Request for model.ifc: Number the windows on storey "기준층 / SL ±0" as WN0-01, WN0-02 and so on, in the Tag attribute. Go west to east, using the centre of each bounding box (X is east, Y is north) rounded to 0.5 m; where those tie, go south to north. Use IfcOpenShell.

First a look at what the model holds.

```python
import ifcopenshell
import ifcopenshell.util.element
import ifcopenshell.util.placement

model = ifcopenshell.open("model.ifc")
print(model.schema)
storey = next(s for s in model.by_type("IfcBuildingStorey") if s.Name == "기준층 / SL ±0")
windows = [e for e in ifcopenshell.util.element.get_decomposition(storey) if e.is_a("IfcWindow")]
for e in sorted(windows, key=lambda e: e.id()):
    origin = ifcopenshell.util.placement.get_local_placement(e.ObjectPlacement)[:3, 3]
    print(e.id(), e.Tag, e.Name, origin.round(2) + 0.0, sep=" | ")
```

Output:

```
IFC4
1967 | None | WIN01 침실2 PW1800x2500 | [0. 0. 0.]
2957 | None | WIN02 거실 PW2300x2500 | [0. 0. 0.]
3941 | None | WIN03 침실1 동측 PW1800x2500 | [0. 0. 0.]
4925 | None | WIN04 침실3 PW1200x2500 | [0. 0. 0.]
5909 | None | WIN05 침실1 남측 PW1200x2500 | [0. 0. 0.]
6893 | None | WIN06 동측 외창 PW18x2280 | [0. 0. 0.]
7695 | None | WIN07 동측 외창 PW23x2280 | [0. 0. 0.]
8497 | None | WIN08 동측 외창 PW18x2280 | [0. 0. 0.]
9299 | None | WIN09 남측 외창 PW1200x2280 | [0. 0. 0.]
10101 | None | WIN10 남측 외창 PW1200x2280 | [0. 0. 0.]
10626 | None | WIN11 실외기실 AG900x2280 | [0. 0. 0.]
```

```python
import ifcopenshell
import ifcopenshell.geom
import ifcopenshell.util.element
import ifcopenshell.util.shape

model = ifcopenshell.open("model.ifc")
settings = ifcopenshell.geom.settings()
settings.set("use-world-coords", True)


def centre(element):
    shape = ifcopenshell.geom.create_shape(settings, element)
    return ifcopenshell.util.shape.get_bbox_centroid(shape.geometry)


storey = next(s for s in model.by_type("IfcBuildingStorey") if s.Name == "기준층 / SL ±0")
windows = [e for e in ifcopenshell.util.element.get_decomposition(storey) if e.is_a("IfcWindow")]

# Insertion points can sit at a corner or the storey origin, so sort by the geometry (in metres).
centres = {e: centre(e) for e in windows}
windows.sort(key=lambda e: (round(centres[e][0] / 0.5), centres[e][1]))

for i, e in enumerate(windows, start=1):
    number = f"WN0-{i:02d}"
    e.Tag = number
    print(e.id(), number)

model.write("model_updated.ifc")
```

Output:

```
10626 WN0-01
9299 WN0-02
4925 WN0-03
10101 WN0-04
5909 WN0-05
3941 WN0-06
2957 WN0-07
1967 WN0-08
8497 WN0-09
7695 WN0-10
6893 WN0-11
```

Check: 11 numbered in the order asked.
